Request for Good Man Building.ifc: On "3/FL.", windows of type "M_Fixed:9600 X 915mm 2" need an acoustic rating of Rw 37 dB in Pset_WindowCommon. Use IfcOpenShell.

First a look at what the model holds.

```python
import ifcopenshell
import ifcopenshell.util.element

model = ifcopenshell.open("Good Man Building.ifc")
print(model.schema)
storey = next(s for s in model.by_type("IfcBuildingStorey") if s.Name == "3/FL.")
windows = [e for e in ifcopenshell.util.element.get_decomposition(storey) if e.is_a("IfcWindow")]
seen = {}
for e in windows:
    element_type = ifcopenshell.util.element.get_type(e)
    key = (element_type.Name if element_type != e and element_type else None, ifcopenshell.util.element.get_pset(e, "Pset_WindowCommon", "AcousticRating"))
    seen[key] = seen.get(key, 0) + 1
for (name, value), count in sorted(seen.items(), key=str):
    print(count, "x", name, "|", value)
```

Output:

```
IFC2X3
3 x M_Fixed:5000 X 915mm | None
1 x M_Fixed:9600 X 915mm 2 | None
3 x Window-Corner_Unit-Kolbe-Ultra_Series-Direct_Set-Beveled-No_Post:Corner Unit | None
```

```python
import ifcopenshell
import ifcopenshell.api.pset
import ifcopenshell.util.element

model = ifcopenshell.open("Good Man Building.ifc")

storey = next(s for s in model.by_type("IfcBuildingStorey") if s.Name == "3/FL.")
windows = [e for e in ifcopenshell.util.element.get_decomposition(storey) if e.is_a("IfcWindow")]

count = 0
for e in windows:
    element_type = ifcopenshell.util.element.get_type(e)
    if element_type in (None, e) or element_type.Name != "M_Fixed:9600 X 915mm 2":
        continue
    # add_pset returns the element's existing set when there is one.
    pset = ifcopenshell.api.pset.add_pset(model, product=e, name="Pset_WindowCommon")
    ifcopenshell.api.pset.edit_pset(model, pset=pset, properties={"AcousticRating": "Rw 37 dB"})
    count += 1

print(count, "windows updated")

model.write("Good Man Building_edited.ifc")
```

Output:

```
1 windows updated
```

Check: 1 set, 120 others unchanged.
